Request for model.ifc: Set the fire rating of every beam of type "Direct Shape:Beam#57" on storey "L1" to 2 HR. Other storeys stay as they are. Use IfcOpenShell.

First a look at what the model holds.

```python
import ifcopenshell
import ifcopenshell.util.element

model = ifcopenshell.open("model.ifc")
print(model.schema)
storey = next(s for s in model.by_type("IfcBuildingStorey") if s.Name == "L1")
beams = [e for e in ifcopenshell.util.element.get_decomposition(storey) if e.is_a("IfcBeam")]
seen = {}
for e in beams:
    element_type = ifcopenshell.util.element.get_type(e)
    key = (element_type.Name if element_type != e and element_type else None, ifcopenshell.util.element.get_pset(e, "Pset_BeamCommon", "FireRating"))
    seen[key] = seen.get(key, 0) + 1
for (name, value), count in sorted(seen.items(), key=str):
    print(count, "x", name, "|", value)
```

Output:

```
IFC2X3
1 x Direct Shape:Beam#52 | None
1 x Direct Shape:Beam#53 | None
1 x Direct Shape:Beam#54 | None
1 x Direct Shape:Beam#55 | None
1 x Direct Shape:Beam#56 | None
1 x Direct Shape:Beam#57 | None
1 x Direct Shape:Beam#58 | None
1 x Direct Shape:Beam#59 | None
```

```python
import ifcopenshell
import ifcopenshell.api.pset
import ifcopenshell.util.element

model = ifcopenshell.open("model.ifc")

storey = next(s for s in model.by_type("IfcBuildingStorey") if s.Name == "L1")
beams = [e for e in ifcopenshell.util.element.get_decomposition(storey) if e.is_a("IfcBeam")]

count = 0
for e in beams:
    element_type = ifcopenshell.util.element.get_type(e)
    if element_type in (None, e) or element_type.Name != "Direct Shape:Beam#57":
        continue
    # add_pset returns the element's existing set when there is one.
    pset = ifcopenshell.api.pset.add_pset(model, product=e, name="Pset_BeamCommon")
    ifcopenshell.api.pset.edit_pset(model, pset=pset, properties={"FireRating": "2 HR"})
    count += 1

print(count, "beams updated")

model.write("model_updated.ifc")
```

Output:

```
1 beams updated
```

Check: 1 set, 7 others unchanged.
